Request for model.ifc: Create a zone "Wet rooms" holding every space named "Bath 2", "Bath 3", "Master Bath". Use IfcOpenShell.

First a look at what the model holds.

```python
import ifcopenshell

model = ifcopenshell.open("model.ifc")
print(model.schema)
seen = {}
for space in model.by_type("IfcSpace"):
    seen[space.LongName] = seen.get(space.LongName, 0) + 1
for name, count in sorted(seen.items(), key=str):
    print(count, "x", name)
print("zones:", [z.Name for z in model.by_type("IfcZone")][:20])
```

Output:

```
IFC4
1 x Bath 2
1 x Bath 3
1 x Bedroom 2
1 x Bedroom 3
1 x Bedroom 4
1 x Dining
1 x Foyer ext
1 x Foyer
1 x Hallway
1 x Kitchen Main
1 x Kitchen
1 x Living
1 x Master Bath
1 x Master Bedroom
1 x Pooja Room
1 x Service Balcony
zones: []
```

```python
import ifcopenshell
import ifcopenshell.api.group
import ifcopenshell.api.root

model = ifcopenshell.open("model.ifc")

names = {"Bath 2", "Bath 3", "Master Bath"}
spaces = [s for s in model.by_type("IfcSpace") if s.LongName in names]

zone = ifcopenshell.api.root.create_entity(model, ifc_class="IfcZone", name="Wet rooms")
ifcopenshell.api.group.assign_group(model, products=spaces, group=zone)
print(len(spaces), "spaces in", zone.Name)

model.write("model_edited.ifc")
```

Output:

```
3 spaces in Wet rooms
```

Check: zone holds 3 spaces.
